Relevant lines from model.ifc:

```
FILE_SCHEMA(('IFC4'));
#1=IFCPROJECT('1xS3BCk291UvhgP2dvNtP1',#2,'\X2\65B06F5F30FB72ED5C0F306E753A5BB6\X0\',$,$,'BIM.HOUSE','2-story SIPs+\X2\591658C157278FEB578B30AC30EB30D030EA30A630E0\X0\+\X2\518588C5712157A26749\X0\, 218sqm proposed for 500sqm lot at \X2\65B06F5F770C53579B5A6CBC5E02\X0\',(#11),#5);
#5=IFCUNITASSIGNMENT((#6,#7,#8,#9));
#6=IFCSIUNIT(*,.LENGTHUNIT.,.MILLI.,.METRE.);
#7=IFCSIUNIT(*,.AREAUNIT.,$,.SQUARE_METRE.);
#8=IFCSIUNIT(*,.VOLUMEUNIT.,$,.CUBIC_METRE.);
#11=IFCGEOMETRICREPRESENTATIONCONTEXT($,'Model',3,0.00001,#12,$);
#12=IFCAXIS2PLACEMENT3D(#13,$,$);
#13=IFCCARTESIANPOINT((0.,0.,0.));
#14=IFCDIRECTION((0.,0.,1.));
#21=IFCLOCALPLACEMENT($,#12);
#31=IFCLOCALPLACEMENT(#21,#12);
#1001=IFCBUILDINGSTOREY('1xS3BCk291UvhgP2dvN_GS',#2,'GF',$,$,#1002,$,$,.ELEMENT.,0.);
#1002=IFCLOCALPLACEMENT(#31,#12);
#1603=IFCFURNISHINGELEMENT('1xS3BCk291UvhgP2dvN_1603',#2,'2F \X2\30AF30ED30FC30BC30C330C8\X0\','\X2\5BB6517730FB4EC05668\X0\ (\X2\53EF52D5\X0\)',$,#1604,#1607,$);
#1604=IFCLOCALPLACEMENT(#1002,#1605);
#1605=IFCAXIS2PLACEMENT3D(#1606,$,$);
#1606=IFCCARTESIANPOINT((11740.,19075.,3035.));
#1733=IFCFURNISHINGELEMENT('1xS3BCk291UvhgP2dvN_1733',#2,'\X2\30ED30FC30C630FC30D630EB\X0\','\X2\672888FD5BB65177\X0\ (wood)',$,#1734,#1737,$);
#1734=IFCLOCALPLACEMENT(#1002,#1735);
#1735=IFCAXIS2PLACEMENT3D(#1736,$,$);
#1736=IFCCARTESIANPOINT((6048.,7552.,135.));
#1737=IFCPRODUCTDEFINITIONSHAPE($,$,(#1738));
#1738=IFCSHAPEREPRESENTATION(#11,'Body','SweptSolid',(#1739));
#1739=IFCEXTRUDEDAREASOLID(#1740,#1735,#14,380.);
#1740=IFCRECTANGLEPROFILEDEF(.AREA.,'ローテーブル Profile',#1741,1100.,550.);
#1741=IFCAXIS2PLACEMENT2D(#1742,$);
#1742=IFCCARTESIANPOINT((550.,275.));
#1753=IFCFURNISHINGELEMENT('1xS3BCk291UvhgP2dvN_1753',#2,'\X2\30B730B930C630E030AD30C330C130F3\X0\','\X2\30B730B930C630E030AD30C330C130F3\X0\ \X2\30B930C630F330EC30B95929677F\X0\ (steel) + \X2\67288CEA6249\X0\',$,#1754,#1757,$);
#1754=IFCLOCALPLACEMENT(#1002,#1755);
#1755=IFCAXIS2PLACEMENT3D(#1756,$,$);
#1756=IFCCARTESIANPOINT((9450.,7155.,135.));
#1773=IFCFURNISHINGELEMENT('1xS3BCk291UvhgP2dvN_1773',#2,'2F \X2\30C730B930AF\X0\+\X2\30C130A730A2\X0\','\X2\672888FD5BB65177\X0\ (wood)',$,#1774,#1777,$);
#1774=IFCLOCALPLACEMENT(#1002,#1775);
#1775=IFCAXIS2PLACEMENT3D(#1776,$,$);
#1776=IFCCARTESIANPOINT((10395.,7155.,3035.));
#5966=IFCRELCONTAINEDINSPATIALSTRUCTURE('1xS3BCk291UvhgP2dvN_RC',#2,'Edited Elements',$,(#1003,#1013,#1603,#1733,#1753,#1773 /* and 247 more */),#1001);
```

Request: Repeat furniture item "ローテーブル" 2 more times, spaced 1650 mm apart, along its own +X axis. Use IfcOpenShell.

```python
import ifcopenshell
import ifcopenshell.api.geometry
import ifcopenshell.api.root
import ifcopenshell.util.element
import ifcopenshell.util.placement

model = ifcopenshell.open("model.ifc")


def reuse_history(source, copy):
    """copy_class also copies each property set's owner history, people and application; keep the originals."""
    for rel in copy.IsDefinedBy:
        if rel.is_a("IfcRelDefinesByProperties") and (history := rel.RelatingPropertyDefinition.OwnerHistory):
            rel.RelatingPropertyDefinition.OwnerHistory = source.OwnerHistory
            ifcopenshell.util.element.remove_deep2(model, history)


source = model.by_guid("1xS3BCk291UvhgP2dvN_1733")
base = ifcopenshell.util.placement.get_local_placement(source.ObjectPlacement)
step = base[:3, 0] * 1650.0

for i in range(1, 3):
    copy = ifcopenshell.api.root.copy_class(model, product=source)
    copy.Representation = ifcopenshell.util.element.copy_deep(
        model, source.Representation, exclude=["IfcGeometricRepresentationContext", "IfcRepresentationMap"]
    )
    reuse_history(source, copy)
    matrix = base.copy()
    matrix[:3, 3] += i * step
    print("added at", matrix[:3, 3].round(3) + 0.0)
    ifcopenshell.api.geometry.edit_object_placement(model, product=copy, matrix=matrix, is_si=False)

model.write("model_v2.ifc")
```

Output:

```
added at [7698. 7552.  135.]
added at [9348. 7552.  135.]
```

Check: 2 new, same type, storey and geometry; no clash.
